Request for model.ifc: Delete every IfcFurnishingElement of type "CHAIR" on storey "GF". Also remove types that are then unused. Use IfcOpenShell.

First a look at what the model holds.

```python
import ifcopenshell
import ifcopenshell.util.element

model = ifcopenshell.open("model.ifc")
print(model.schema)
storey = next(s for s in model.by_type("IfcBuildingStorey") if s.Name == "GF")
furniture = [e for e in ifcopenshell.util.element.get_decomposition(storey) if e.is_a("IfcFurnishingElement")]
seen = {}
for e in furniture:
    element_type = ifcopenshell.util.element.get_type(e)
    name = element_type.Name if element_type not in (None, e) else None
    seen[name] = seen.get(name, 0) + 1
for name, count in sorted(seen.items(), key=str):
    print(count, "x", name)
```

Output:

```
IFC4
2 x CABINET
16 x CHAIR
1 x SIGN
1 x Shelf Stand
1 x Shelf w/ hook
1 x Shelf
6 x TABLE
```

```python
import ifcopenshell
import ifcopenshell.api.root
import ifcopenshell.util.element

model = ifcopenshell.open("model.ifc")

storey = next(s for s in model.by_type("IfcBuildingStorey") if s.Name == "GF")
furniture = [e for e in ifcopenshell.util.element.get_decomposition(storey) if e.is_a("IfcFurnishingElement")]
targets = [e for e in furniture if (t := ifcopenshell.util.element.get_type(e)) not in (None, e) and t.Name == "CHAIR"]
types = {ifcopenshell.util.element.get_type(e) for e in targets} - {None, *targets}

for e in targets:
    ifcopenshell.api.root.remove_product(model, product=e)
print(len(targets), "removed")

unused = [t for t in types if not ifcopenshell.util.element.get_types(t)]
for t in unused:
    ifcopenshell.api.root.remove_product(model, product=t)
print(len(unused), "unused types removed")

model.write("model_updated.ifc")
```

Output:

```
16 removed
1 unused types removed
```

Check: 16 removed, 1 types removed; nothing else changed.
